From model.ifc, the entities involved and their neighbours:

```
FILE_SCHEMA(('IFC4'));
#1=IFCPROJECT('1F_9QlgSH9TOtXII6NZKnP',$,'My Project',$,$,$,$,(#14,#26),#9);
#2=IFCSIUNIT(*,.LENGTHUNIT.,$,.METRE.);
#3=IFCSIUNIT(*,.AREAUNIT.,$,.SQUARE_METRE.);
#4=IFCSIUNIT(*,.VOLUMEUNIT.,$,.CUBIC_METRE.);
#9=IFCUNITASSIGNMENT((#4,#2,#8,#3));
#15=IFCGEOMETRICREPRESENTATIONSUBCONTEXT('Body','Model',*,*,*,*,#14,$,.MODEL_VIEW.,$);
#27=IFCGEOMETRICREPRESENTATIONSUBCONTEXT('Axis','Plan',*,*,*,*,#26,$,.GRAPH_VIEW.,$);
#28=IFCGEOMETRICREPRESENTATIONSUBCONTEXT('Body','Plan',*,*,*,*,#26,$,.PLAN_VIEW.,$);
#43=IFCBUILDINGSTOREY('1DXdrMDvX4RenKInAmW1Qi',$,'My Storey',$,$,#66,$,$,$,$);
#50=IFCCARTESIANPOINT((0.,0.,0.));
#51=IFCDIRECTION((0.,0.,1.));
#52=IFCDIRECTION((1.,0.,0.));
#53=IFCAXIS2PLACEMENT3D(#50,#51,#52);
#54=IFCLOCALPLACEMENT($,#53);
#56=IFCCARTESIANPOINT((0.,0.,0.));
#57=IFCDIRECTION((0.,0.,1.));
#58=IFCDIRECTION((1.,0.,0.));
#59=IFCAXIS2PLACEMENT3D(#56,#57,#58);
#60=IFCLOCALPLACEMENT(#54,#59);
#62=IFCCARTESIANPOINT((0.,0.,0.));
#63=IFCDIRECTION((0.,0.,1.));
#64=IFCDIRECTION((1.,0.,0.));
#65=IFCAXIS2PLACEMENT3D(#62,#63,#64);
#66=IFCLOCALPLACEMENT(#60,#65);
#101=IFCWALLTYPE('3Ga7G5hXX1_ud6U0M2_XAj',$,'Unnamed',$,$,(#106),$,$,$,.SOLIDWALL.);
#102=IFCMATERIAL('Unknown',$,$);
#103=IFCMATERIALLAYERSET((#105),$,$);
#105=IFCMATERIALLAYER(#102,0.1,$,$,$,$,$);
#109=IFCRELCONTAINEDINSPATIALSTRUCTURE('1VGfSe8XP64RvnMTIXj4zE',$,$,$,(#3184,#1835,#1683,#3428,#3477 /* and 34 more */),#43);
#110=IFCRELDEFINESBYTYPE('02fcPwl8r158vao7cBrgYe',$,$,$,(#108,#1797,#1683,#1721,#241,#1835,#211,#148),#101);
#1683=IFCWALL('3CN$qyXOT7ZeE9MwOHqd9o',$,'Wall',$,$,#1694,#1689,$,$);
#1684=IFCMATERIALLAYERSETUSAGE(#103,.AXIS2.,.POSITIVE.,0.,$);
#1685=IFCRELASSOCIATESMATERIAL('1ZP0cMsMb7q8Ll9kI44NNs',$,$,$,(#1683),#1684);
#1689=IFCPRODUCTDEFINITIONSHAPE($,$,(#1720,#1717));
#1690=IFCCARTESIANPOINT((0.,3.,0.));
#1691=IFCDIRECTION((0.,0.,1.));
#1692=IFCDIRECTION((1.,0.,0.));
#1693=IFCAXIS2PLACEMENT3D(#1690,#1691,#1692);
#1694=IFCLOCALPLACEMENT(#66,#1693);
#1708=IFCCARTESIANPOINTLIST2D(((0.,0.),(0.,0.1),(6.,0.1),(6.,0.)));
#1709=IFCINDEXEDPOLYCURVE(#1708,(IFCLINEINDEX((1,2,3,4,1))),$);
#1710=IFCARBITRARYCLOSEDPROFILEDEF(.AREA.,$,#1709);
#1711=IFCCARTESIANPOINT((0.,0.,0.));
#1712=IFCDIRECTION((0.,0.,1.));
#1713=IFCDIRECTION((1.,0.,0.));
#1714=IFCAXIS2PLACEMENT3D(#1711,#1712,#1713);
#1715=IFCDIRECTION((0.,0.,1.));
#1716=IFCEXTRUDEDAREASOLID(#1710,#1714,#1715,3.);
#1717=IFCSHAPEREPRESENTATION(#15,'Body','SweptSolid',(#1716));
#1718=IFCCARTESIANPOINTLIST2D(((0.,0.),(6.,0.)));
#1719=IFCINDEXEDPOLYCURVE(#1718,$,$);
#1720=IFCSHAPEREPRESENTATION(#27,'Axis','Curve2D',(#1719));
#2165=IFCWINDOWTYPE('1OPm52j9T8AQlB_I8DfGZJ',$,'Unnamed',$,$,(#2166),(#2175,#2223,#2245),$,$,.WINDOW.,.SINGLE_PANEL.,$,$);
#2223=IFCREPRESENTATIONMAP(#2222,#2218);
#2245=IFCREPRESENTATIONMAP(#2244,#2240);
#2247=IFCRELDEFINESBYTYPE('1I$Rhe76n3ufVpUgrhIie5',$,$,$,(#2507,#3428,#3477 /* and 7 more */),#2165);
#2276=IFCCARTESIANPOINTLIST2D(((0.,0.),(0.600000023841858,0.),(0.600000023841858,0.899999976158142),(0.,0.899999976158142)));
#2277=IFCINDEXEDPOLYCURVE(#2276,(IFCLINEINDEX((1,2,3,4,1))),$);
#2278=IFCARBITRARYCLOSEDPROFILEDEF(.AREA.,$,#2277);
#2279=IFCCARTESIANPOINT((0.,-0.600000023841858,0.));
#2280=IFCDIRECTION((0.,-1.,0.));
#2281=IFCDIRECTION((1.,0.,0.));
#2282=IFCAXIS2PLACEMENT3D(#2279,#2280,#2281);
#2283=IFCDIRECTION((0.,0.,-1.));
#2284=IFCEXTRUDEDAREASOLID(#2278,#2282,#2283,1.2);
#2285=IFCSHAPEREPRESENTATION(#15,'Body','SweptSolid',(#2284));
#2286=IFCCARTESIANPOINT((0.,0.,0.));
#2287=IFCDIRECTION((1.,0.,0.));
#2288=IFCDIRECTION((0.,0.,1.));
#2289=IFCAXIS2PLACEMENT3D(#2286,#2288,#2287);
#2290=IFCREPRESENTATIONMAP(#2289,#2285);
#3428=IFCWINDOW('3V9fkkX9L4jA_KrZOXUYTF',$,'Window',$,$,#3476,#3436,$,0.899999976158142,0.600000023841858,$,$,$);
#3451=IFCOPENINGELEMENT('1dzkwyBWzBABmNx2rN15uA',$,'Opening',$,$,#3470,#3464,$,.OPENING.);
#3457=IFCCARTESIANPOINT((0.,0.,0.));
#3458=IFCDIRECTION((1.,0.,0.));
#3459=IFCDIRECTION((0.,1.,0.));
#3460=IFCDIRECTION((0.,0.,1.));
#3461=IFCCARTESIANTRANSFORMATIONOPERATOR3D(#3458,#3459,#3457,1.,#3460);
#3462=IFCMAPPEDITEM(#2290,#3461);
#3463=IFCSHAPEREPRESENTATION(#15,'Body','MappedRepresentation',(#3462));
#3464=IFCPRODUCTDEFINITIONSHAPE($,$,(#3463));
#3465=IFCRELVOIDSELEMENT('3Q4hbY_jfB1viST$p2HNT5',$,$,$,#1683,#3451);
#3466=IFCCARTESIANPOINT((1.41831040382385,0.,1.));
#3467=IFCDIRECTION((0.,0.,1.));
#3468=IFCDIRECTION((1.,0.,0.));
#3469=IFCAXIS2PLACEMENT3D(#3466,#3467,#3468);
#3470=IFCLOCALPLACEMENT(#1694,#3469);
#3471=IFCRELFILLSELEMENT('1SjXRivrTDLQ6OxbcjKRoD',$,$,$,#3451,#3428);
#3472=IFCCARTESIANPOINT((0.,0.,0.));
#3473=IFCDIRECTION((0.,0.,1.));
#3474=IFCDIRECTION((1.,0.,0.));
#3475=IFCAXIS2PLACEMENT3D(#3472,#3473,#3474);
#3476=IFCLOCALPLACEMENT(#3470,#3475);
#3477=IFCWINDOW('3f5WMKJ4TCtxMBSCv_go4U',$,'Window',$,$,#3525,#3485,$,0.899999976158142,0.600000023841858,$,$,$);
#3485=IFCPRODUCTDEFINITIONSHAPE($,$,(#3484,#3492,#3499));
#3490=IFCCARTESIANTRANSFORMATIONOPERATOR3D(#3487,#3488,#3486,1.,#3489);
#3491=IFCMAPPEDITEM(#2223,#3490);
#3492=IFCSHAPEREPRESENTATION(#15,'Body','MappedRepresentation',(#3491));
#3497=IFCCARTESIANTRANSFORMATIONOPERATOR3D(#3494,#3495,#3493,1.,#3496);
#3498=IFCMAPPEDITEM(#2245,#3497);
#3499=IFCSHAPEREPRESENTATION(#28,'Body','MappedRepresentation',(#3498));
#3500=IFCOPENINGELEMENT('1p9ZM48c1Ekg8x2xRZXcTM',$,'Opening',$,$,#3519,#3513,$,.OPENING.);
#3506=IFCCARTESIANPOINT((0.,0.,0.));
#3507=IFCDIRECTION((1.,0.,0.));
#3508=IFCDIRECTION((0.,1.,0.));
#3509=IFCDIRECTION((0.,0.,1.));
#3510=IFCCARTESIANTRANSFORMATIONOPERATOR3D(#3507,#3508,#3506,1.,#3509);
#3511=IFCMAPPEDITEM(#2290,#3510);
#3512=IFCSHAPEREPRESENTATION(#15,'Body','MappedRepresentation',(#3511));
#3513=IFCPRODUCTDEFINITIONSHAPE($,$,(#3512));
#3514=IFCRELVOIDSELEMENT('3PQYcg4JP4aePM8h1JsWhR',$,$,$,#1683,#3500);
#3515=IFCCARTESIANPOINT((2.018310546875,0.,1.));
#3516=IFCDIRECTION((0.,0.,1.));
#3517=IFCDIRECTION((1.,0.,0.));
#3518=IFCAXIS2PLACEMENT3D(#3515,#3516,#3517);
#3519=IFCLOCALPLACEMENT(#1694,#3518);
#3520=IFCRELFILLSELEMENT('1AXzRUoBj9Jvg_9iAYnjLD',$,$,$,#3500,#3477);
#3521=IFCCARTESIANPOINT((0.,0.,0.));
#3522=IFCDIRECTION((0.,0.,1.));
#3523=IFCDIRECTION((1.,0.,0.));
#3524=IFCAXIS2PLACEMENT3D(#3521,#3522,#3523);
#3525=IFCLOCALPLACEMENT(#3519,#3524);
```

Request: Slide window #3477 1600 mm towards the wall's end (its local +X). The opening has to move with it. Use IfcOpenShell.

```python
import ifcopenshell
import ifcopenshell.api.geometry
import ifcopenshell.util.placement
import ifcopenshell.util.unit

model = ifcopenshell.open("model.ifc")
unit_scale = ifcopenshell.util.unit.calculate_unit_scale(model)

window = model.by_guid("3f5WMKJ4TCtxMBSCv_go4U")
opening = window.FillsVoids[0].RelatingOpeningElement
wall = opening.VoidsElements[0].RelatingBuildingElement

wall_matrix = ifcopenshell.util.placement.get_local_placement(wall.ObjectPlacement)
shift = wall_matrix[:3, 0] * 1.6 / unit_scale
before = ifcopenshell.util.placement.get_local_placement(window.ObjectPlacement)[:3, 3].copy()

# The window is placed relative to its opening, so it follows when the opening moves.
matrix = ifcopenshell.util.placement.get_local_placement(opening.ObjectPlacement)
matrix[:3, 3] += shift
ifcopenshell.api.geometry.edit_object_placement(
    model, product=opening, matrix=matrix, is_si=False, should_transform_children=True
)

after = ifcopenshell.util.placement.get_local_placement(window.ObjectPlacement)[:3, 3]
print("window moved by", (after - before).round(3) + 0.0)

model.write("model-out.ifc")
```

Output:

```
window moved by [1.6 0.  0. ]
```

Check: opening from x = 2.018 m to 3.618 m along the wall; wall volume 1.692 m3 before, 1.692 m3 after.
